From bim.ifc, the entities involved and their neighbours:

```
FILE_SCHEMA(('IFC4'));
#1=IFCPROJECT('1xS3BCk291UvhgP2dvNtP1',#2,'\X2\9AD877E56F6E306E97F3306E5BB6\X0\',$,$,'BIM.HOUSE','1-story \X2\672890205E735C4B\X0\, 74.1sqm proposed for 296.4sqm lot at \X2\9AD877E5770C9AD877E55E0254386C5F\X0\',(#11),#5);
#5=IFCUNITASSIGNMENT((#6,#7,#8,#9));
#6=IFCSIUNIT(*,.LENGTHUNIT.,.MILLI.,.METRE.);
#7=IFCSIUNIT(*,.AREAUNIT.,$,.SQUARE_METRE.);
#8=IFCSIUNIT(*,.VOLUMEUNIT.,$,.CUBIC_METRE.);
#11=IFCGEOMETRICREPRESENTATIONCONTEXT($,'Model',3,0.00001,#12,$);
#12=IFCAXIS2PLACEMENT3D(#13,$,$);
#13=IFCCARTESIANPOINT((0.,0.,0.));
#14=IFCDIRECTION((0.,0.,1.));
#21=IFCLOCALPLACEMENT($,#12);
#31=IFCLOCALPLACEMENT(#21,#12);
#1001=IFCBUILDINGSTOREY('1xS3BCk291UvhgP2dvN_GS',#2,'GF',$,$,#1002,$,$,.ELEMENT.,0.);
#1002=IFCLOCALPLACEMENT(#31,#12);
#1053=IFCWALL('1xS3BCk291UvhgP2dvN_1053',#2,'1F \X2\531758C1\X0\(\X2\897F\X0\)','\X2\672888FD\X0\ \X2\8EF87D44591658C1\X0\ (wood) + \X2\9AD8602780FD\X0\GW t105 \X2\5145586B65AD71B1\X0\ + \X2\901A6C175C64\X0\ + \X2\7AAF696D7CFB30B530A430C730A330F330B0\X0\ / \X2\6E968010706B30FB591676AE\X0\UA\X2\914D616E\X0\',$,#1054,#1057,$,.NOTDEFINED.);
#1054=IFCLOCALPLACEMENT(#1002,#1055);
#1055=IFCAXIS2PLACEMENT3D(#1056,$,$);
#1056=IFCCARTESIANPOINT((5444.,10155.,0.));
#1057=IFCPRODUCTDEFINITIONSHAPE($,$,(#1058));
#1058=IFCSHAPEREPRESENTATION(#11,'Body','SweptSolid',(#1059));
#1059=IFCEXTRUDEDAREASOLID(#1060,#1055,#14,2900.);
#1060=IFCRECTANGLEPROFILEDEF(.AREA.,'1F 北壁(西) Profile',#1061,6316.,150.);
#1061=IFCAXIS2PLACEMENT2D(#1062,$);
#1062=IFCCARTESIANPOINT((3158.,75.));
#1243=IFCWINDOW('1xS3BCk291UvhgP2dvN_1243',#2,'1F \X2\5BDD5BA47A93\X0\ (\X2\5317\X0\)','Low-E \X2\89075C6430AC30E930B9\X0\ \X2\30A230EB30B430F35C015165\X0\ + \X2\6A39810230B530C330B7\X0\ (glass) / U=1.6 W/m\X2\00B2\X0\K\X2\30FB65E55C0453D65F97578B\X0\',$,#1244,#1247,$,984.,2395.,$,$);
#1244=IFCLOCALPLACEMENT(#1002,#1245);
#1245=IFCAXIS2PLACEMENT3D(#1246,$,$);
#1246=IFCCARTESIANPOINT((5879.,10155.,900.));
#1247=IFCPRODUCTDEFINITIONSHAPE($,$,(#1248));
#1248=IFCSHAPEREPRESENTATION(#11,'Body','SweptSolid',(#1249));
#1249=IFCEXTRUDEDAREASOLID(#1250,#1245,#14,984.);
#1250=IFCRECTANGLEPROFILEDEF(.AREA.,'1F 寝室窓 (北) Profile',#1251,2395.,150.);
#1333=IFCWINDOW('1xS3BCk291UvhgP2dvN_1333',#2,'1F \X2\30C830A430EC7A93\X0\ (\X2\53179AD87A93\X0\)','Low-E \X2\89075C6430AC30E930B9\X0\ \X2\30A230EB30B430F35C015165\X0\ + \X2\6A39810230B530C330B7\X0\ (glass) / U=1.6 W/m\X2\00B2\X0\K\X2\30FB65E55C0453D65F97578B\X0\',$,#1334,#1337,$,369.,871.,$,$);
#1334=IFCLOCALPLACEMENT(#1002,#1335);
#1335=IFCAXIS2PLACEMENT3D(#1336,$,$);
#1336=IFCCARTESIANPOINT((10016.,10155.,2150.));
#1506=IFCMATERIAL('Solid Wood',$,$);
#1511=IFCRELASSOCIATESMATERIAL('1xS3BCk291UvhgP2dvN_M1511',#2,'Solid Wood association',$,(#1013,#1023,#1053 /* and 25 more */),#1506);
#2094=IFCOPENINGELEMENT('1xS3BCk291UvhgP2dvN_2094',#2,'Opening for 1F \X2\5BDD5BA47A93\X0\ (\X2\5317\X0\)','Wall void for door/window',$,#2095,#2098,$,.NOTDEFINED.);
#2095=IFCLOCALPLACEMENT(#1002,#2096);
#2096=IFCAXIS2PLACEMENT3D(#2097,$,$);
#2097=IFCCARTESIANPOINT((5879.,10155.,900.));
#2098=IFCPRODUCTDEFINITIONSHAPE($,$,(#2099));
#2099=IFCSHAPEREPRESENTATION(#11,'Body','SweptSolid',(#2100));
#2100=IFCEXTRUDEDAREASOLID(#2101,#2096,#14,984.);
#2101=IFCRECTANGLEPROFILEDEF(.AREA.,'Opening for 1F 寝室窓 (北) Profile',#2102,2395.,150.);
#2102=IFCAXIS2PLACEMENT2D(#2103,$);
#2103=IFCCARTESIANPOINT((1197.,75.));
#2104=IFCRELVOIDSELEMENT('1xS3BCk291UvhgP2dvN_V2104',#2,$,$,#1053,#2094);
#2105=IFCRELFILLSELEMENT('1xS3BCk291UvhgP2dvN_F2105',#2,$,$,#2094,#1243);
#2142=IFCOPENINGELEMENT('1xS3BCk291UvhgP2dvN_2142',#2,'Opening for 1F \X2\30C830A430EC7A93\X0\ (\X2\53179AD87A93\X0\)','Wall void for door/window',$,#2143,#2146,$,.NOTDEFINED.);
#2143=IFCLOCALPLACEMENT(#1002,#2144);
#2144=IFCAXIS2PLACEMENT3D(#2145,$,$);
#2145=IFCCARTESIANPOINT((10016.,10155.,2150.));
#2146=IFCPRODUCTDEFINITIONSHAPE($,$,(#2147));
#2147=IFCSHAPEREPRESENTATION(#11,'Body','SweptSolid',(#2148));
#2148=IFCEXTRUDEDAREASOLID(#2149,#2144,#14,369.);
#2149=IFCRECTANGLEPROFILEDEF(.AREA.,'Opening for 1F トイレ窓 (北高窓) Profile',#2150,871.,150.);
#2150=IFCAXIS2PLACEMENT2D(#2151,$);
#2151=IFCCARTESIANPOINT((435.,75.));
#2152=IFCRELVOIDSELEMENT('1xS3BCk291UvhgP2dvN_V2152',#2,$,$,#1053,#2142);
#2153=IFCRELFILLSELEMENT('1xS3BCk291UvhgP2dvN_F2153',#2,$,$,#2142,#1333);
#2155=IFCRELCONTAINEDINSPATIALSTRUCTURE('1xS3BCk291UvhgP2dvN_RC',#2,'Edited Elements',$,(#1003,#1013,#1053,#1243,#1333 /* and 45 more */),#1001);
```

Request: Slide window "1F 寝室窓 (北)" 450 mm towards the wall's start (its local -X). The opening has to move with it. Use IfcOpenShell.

```python
import ifcopenshell
import ifcopenshell.api.geometry
import ifcopenshell.util.placement
import ifcopenshell.util.unit

model = ifcopenshell.open("bim.ifc")
unit_scale = ifcopenshell.util.unit.calculate_unit_scale(model)

window = model.by_guid("1xS3BCk291UvhgP2dvN_1243")
opening = window.FillsVoids[0].RelatingOpeningElement
wall = opening.VoidsElements[0].RelatingBuildingElement

wall_matrix = ifcopenshell.util.placement.get_local_placement(wall.ObjectPlacement)
shift = wall_matrix[:3, 0] * -0.45 / unit_scale
before = ifcopenshell.util.placement.get_local_placement(window.ObjectPlacement)[:3, 3].copy()

# The window is not placed relative to its opening, so move both.
for product in (opening, window):
    matrix = ifcopenshell.util.placement.get_local_placement(product.ObjectPlacement)
    matrix[:3, 3] += shift
    ifcopenshell.api.geometry.edit_object_placement(model, product=product, matrix=matrix, is_si=False)

after = ifcopenshell.util.placement.get_local_placement(window.ObjectPlacement)[:3, 3]
print("window moved by", (after - before).round(3) + 0.0)

model.write("bim_edited.ifc")
```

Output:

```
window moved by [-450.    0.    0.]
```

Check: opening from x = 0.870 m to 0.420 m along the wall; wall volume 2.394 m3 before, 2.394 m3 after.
